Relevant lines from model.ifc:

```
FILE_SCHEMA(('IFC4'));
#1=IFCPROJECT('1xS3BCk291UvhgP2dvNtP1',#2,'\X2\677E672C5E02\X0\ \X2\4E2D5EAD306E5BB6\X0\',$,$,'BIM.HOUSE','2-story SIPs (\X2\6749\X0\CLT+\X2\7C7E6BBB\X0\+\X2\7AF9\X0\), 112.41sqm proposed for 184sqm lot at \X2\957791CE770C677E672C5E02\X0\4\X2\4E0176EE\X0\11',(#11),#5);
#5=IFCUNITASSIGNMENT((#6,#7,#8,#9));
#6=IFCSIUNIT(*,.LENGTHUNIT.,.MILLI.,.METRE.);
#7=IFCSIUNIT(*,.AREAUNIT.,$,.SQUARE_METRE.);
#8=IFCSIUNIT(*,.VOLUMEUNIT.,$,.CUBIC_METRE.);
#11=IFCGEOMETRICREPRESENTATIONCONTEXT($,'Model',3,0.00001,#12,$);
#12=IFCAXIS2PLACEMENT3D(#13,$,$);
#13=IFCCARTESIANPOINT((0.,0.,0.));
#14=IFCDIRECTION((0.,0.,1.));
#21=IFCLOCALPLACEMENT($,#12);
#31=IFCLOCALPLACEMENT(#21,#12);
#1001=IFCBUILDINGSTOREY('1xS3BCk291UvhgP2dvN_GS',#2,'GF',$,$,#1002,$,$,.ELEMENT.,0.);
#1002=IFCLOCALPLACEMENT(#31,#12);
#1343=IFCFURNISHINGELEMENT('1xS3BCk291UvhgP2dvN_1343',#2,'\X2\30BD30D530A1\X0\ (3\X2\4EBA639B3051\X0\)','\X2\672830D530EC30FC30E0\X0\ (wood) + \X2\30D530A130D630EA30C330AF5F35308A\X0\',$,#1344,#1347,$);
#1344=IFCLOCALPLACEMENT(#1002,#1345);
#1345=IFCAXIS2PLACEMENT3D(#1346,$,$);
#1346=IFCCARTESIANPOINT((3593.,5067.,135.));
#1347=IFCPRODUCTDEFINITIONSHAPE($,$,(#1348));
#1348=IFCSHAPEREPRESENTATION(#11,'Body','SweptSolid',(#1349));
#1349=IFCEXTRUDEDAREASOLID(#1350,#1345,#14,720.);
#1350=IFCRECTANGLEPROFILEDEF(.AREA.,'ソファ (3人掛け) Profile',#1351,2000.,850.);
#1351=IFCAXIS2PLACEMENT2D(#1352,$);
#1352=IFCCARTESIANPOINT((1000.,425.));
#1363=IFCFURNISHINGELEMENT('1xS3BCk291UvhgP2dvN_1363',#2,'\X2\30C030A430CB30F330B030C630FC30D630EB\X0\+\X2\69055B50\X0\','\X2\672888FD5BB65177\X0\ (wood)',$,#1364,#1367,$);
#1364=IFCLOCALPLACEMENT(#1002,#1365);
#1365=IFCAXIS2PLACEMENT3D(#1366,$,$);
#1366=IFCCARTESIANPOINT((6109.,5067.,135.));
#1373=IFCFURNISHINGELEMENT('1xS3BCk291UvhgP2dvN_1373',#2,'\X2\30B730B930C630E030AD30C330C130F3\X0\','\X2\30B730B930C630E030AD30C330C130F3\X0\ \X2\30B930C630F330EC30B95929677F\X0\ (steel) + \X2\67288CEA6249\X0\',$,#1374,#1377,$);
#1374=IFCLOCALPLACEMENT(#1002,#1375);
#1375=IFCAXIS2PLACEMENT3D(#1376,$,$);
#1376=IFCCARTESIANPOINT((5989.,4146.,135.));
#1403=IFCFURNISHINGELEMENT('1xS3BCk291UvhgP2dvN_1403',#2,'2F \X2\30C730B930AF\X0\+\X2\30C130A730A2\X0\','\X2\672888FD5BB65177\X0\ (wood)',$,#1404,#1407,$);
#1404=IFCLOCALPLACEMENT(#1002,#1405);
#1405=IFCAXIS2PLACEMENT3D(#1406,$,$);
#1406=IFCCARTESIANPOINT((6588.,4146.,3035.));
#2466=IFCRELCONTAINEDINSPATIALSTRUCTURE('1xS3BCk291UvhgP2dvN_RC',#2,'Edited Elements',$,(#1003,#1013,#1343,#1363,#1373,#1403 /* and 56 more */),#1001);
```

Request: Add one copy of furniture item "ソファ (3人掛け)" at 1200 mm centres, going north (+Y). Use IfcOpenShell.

```python
import numpy as np
import ifcopenshell
import ifcopenshell.api.geometry
import ifcopenshell.api.root
import ifcopenshell.util.element
import ifcopenshell.util.placement

model = ifcopenshell.open("model.ifc")


def reuse_history(source, copy):
    """copy_class also copies each property set's owner history, people and application; keep the originals."""
    for rel in copy.IsDefinedBy:
        if rel.is_a("IfcRelDefinesByProperties") and (history := rel.RelatingPropertyDefinition.OwnerHistory):
            rel.RelatingPropertyDefinition.OwnerHistory = source.OwnerHistory
            ifcopenshell.util.element.remove_deep2(model, history)


source = model.by_id(1343)
base = ifcopenshell.util.placement.get_local_placement(source.ObjectPlacement)
step = np.array([0.0, 1.0, 0.0]) * 1200.0

for i in range(1, 2):
    copy = ifcopenshell.api.root.copy_class(model, product=source)
    copy.Representation = ifcopenshell.util.element.copy_deep(
        model, source.Representation, exclude=["IfcGeometricRepresentationContext", "IfcRepresentationMap"]
    )
    reuse_history(source, copy)
    matrix = base.copy()
    matrix[:3, 3] += i * step
    print("added at", matrix[:3, 3].round(3) + 0.0)
    ifcopenshell.api.geometry.edit_object_placement(model, product=copy, matrix=matrix, is_si=False)

model.write("model-out.ifc")
```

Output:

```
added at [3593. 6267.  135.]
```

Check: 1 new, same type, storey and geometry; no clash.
